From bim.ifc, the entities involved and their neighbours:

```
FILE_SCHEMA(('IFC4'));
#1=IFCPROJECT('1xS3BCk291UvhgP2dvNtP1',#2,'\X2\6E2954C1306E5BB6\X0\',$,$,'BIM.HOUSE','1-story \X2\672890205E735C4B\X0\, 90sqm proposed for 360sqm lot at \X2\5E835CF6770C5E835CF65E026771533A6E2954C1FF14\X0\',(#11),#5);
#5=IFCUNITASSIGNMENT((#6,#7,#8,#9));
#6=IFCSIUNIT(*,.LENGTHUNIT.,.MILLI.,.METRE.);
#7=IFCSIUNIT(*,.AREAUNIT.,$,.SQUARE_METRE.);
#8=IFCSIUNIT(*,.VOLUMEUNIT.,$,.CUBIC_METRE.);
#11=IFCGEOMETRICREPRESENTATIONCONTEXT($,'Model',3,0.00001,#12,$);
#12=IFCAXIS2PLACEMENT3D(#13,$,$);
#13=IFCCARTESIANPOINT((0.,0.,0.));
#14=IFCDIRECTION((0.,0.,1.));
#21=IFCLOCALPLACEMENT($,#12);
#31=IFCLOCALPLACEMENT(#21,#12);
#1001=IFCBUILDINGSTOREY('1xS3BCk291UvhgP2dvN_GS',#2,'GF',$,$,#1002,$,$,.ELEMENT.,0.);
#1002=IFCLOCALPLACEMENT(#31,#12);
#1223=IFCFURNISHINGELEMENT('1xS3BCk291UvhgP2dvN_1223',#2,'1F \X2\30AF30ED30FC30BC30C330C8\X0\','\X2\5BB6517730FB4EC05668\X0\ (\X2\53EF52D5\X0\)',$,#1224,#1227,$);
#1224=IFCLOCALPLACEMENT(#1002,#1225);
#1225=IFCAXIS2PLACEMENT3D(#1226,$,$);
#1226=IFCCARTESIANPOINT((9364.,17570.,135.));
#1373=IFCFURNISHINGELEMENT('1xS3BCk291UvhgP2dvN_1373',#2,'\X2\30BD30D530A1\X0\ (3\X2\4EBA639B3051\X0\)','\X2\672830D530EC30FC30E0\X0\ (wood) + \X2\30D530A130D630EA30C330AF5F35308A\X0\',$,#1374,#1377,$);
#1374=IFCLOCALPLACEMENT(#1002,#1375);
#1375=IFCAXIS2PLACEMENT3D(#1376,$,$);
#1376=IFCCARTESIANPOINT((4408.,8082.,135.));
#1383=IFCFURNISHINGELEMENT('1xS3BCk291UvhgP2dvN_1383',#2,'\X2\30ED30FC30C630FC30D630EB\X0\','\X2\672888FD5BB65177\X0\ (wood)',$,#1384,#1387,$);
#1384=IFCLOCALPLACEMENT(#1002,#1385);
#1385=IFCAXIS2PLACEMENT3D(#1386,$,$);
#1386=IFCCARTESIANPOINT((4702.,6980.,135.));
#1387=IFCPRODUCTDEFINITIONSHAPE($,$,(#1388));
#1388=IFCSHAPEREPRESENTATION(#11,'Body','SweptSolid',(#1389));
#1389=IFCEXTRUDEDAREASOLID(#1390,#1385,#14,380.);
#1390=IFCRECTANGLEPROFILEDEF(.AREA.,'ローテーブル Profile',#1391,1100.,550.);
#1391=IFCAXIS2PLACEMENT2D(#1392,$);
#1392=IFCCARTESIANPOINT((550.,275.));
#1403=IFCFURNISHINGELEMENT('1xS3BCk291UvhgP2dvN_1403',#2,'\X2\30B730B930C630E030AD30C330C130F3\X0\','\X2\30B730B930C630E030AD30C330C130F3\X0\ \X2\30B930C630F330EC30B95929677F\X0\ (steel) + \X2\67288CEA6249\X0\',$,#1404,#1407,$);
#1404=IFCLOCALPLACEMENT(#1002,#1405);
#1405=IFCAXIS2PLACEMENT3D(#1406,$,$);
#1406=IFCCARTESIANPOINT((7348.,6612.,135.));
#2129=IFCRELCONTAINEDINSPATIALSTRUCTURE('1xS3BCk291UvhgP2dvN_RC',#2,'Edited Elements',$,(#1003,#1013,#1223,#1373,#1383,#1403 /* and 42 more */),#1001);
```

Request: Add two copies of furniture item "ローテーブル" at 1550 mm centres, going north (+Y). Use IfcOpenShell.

```python
import numpy as np
import ifcopenshell
import ifcopenshell.api.geometry
import ifcopenshell.api.root
import ifcopenshell.util.element
import ifcopenshell.util.placement
import ifcopenshell.util.unit

model = ifcopenshell.open("bim.ifc")
unit_scale = ifcopenshell.util.unit.calculate_unit_scale(model)


def reuse_history(source, copy):
    """copy_class also copies each property set's owner history, people and application; keep the originals."""
    for rel in copy.IsDefinedBy:
        if rel.is_a("IfcRelDefinesByProperties") and (history := rel.RelatingPropertyDefinition.OwnerHistory):
            rel.RelatingPropertyDefinition.OwnerHistory = source.OwnerHistory
            ifcopenshell.util.element.remove_deep2(model, history)


source = model.by_guid("1xS3BCk291UvhgP2dvN_1383")
base = ifcopenshell.util.placement.get_local_placement(source.ObjectPlacement)
step = np.array([0.0, 1.0, 0.0]) * 1.55 / unit_scale

for i in range(1, 3):
    copy = ifcopenshell.api.root.copy_class(model, product=source)
    copy.Representation = ifcopenshell.util.element.copy_deep(
        model, source.Representation, exclude=["IfcGeometricRepresentationContext", "IfcRepresentationMap"]
    )
    reuse_history(source, copy)
    matrix = base.copy()
    matrix[:3, 3] += i * step
    print("added at", matrix[:3, 3].round(3) + 0.0)
    ifcopenshell.api.geometry.edit_object_placement(model, product=copy, matrix=matrix, is_si=False)

model.write("bim_edited.ifc")
```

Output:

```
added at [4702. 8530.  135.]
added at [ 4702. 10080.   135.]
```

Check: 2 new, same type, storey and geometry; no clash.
